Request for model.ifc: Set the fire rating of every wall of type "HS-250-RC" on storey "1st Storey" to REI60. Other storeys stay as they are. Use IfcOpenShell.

First a look at what the model holds.

```python
import ifcopenshell
import ifcopenshell.util.element

model = ifcopenshell.open("model.ifc")
print(model.schema)
storey = next(s for s in model.by_type("IfcBuildingStorey") if s.Name == "1st Storey")
walls = [e for e in ifcopenshell.util.element.get_decomposition(storey) if e.is_a("IfcWall")]
seen = {}
for e in walls:
    element_type = ifcopenshell.util.element.get_type(e)
    key = (element_type.Name if element_type != e and element_type else None, ifcopenshell.util.element.get_pset(e, "Pset_WallCommon", "FireRating"))
    seen[key] = seen.get(key, 0) + 1
for (name, value), count in sorted(seen.items(), key=str):
    print(count, "x", name, "|", value)
```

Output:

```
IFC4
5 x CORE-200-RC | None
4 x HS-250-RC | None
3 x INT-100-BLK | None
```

```python
import ifcopenshell
import ifcopenshell.api.pset
import ifcopenshell.util.element

model = ifcopenshell.open("model.ifc")

storey = next(s for s in model.by_type("IfcBuildingStorey") if s.Name == "1st Storey")
walls = [e for e in ifcopenshell.util.element.get_decomposition(storey) if e.is_a("IfcWall")]

count = 0
for e in walls:
    element_type = ifcopenshell.util.element.get_type(e)
    if element_type in (None, e) or element_type.Name != "HS-250-RC":
        continue
    # add_pset returns the element's existing set when there is one.
    pset = ifcopenshell.api.pset.add_pset(model, product=e, name="Pset_WallCommon")
    ifcopenshell.api.pset.edit_pset(model, pset=pset, properties={"FireRating": "REI60"})
    count += 1

print(count, "walls updated")

model.write("model_updated.ifc")
```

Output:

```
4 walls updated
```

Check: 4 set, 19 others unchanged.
